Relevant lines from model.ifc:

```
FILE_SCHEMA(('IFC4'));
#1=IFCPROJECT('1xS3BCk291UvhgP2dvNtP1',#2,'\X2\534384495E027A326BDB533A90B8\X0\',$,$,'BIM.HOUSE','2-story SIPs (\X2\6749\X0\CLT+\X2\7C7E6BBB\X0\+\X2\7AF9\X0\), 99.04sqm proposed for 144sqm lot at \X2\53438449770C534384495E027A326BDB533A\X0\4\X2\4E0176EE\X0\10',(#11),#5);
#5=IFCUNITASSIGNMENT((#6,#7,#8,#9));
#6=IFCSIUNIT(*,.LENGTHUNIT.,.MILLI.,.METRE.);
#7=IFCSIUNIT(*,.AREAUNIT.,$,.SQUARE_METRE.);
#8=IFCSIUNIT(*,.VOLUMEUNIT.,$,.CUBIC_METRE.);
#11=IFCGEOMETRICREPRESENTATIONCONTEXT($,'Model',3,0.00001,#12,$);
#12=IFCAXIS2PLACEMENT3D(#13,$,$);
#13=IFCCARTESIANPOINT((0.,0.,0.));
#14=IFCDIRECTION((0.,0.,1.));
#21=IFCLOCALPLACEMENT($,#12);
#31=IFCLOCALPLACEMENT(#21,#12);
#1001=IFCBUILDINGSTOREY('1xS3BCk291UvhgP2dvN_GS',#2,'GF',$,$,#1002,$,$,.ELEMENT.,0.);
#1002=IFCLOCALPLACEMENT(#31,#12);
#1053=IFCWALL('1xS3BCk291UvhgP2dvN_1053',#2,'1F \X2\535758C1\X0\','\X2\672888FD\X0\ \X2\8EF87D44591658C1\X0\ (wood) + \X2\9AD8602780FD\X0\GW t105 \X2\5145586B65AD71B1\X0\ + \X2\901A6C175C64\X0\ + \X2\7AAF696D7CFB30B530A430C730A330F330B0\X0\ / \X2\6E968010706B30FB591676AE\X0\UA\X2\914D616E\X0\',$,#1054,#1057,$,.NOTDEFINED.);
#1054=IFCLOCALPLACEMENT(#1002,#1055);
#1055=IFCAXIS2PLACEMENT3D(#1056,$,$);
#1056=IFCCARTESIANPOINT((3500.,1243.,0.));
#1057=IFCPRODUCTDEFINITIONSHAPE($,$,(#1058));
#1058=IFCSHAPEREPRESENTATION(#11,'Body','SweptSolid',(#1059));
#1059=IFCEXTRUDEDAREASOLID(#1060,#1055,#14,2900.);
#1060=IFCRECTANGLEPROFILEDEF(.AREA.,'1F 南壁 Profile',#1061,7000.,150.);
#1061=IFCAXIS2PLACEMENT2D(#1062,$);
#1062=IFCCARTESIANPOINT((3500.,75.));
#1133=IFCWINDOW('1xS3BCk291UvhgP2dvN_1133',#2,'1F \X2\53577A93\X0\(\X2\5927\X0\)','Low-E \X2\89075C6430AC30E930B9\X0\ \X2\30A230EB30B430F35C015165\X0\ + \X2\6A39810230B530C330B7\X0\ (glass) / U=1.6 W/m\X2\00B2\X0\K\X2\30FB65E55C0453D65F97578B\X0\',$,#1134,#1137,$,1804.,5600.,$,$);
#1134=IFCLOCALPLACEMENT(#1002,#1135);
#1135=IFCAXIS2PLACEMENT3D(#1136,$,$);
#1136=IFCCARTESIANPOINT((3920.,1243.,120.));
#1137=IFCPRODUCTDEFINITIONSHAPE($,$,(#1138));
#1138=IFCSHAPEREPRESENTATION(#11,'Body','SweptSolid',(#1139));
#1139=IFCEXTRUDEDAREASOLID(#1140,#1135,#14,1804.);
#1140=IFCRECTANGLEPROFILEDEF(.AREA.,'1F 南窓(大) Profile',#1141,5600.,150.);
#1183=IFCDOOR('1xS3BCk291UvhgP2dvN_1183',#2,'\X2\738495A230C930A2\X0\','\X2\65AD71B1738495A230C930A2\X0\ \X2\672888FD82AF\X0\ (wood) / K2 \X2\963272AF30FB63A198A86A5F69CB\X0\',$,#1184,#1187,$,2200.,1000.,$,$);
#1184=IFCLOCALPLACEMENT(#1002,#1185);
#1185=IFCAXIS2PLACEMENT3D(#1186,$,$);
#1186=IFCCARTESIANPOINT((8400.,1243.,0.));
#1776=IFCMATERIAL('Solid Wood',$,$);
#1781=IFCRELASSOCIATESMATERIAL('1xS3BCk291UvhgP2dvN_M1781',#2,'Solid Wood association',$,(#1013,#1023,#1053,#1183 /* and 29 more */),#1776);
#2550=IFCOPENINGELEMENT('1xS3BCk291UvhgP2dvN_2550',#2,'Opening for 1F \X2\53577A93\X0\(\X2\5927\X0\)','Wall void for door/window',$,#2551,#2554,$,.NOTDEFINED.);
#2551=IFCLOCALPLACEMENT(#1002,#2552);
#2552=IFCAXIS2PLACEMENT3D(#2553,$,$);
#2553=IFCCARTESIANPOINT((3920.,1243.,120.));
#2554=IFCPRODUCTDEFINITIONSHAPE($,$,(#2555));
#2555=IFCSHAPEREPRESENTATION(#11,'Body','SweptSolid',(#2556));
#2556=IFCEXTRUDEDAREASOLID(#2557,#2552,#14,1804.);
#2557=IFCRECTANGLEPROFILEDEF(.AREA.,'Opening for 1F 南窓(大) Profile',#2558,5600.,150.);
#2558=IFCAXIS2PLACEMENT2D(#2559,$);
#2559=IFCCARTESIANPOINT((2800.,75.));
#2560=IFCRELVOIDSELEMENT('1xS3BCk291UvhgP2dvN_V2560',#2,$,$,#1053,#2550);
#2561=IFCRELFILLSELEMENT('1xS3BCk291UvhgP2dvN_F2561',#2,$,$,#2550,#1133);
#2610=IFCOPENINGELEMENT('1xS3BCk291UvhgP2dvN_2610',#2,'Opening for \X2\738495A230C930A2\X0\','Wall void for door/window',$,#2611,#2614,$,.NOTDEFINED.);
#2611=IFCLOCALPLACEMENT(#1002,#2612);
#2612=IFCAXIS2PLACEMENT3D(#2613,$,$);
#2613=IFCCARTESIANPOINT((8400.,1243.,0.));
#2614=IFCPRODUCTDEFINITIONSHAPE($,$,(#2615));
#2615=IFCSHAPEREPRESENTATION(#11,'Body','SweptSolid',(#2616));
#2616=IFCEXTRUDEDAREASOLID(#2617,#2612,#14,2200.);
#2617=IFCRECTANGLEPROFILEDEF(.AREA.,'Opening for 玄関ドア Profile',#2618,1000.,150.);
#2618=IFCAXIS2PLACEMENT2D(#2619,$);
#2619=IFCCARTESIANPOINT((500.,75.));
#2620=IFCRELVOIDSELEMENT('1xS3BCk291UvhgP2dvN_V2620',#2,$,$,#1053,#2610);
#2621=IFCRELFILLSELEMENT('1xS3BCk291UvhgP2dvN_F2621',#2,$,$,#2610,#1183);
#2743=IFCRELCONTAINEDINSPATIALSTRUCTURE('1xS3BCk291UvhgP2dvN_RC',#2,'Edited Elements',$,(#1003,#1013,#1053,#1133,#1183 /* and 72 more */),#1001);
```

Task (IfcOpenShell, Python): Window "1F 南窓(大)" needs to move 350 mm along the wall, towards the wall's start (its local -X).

```python
import ifcopenshell
import ifcopenshell.api.geometry
import ifcopenshell.util.placement

model = ifcopenshell.open("model.ifc")

window = model.by_guid("1xS3BCk291UvhgP2dvN_1133")
opening = window.FillsVoids[0].RelatingOpeningElement
wall = opening.VoidsElements[0].RelatingBuildingElement

wall_matrix = ifcopenshell.util.placement.get_local_placement(wall.ObjectPlacement)
shift = wall_matrix[:3, 0] * -350.0
before = ifcopenshell.util.placement.get_local_placement(window.ObjectPlacement)[:3, 3].copy()

# The window is not placed relative to its opening, so move both.
for product in (opening, window):
    matrix = ifcopenshell.util.placement.get_local_placement(product.ObjectPlacement)
    matrix[:3, 3] += shift
    ifcopenshell.api.geometry.edit_object_placement(model, product=product, matrix=matrix, is_si=False)

after = ifcopenshell.util.placement.get_local_placement(window.ObjectPlacement)[:3, 3]
print("window moved by", (after - before).round(3) + 0.0)

model.write("model-out.ifc")
```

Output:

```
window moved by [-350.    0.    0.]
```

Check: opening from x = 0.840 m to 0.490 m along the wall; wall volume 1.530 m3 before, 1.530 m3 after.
